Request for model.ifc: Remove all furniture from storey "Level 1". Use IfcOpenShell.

First a look at what the model holds.

```python
import ifcopenshell
import ifcopenshell.util.element

model = ifcopenshell.open("model.ifc")
print(model.schema)
storey = next(s for s in model.by_type("IfcBuildingStorey") if s.Name == "Level 1")
furniture = [e for e in ifcopenshell.util.element.get_decomposition(storey) if e.is_a("IfcFurnishingElement")]
seen = {}
for e in furniture:
    element_type = ifcopenshell.util.element.get_type(e)
    name = element_type.Name if element_type not in (None, e) else None
    seen[name] = seen.get(name, 0) + 1
for name, count in sorted(seen.items(), key=str):
    print(count, "x", name)
```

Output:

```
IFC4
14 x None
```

```python
import ifcopenshell
import ifcopenshell.api.root
import ifcopenshell.util.element

model = ifcopenshell.open("model.ifc")

storey = next(s for s in model.by_type("IfcBuildingStorey") if s.Name == "Level 1")
furniture = [e for e in ifcopenshell.util.element.get_decomposition(storey) if e.is_a("IfcFurnishingElement")]

for e in furniture:
    ifcopenshell.api.root.remove_product(model, product=e)
print(len(furniture), "removed")

model.write("model_v2.ifc")
```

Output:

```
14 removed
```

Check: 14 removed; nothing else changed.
